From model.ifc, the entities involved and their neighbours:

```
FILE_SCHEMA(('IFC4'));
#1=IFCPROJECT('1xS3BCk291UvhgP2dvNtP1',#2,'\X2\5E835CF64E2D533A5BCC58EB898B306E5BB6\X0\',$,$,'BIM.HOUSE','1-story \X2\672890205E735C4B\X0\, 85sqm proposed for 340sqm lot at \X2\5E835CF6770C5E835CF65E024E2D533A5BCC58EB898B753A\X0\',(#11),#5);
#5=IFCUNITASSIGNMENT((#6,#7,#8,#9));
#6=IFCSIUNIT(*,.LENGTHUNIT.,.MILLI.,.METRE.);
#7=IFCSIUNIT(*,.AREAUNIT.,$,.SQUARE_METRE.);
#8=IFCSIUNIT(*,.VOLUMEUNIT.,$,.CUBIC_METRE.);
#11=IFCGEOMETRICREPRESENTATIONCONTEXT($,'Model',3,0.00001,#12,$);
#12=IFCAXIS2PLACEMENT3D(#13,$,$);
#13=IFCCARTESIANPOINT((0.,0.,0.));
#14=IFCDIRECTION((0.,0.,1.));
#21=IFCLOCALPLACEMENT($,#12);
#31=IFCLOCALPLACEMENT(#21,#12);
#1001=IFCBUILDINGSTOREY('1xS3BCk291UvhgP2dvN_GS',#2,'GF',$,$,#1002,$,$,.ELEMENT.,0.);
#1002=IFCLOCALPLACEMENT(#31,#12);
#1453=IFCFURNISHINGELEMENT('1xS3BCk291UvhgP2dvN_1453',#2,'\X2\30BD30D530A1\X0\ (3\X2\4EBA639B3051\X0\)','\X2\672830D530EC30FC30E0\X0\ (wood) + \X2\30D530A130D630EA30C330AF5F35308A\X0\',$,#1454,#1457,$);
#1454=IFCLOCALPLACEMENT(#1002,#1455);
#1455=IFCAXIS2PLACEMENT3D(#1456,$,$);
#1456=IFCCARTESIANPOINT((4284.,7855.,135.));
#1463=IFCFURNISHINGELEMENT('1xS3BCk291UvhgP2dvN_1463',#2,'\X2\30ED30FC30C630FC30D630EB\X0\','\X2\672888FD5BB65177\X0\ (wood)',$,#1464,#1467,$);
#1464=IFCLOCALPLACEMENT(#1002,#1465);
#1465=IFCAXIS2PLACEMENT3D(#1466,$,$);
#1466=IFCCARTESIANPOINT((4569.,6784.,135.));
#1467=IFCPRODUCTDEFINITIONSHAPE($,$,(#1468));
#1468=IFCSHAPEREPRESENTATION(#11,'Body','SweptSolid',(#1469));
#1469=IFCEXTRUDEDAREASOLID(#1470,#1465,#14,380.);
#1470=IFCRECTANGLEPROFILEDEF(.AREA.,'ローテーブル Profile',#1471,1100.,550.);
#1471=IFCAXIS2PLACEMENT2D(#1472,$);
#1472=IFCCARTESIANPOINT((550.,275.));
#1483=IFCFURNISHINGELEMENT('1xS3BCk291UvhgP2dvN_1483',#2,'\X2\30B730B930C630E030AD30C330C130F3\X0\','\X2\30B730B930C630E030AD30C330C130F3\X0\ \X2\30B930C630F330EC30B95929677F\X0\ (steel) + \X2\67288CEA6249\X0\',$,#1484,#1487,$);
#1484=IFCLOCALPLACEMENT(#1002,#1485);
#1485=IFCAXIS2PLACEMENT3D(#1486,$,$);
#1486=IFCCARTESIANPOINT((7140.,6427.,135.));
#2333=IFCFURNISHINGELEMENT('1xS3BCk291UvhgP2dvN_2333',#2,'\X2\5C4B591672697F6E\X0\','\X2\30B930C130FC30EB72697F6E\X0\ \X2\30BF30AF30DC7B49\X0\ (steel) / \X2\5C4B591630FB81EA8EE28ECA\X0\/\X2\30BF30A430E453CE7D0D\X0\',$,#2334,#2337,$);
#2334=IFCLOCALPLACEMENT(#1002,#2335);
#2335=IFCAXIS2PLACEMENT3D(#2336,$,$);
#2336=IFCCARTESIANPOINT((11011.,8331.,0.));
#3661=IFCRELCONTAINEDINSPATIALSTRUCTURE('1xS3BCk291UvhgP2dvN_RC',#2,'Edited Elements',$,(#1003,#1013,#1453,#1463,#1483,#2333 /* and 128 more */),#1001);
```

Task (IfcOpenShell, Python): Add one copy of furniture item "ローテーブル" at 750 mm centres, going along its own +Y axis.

```python
import ifcopenshell
import ifcopenshell.api.geometry
import ifcopenshell.api.root
import ifcopenshell.util.element
import ifcopenshell.util.placement

model = ifcopenshell.open("model.ifc")


def reuse_history(source, copy):
    """copy_class also copies each property set's owner history, people and application; keep the originals."""
    for rel in copy.IsDefinedBy:
        if rel.is_a("IfcRelDefinesByProperties") and (history := rel.RelatingPropertyDefinition.OwnerHistory):
            rel.RelatingPropertyDefinition.OwnerHistory = source.OwnerHistory
            ifcopenshell.util.element.remove_deep2(model, history)


source = model.by_guid("1xS3BCk291UvhgP2dvN_1463")
base = ifcopenshell.util.placement.get_local_placement(source.ObjectPlacement)
step = base[:3, 1] * 750.0

for i in range(1, 2):
    copy = ifcopenshell.api.root.copy_class(model, product=source)
    copy.Representation = ifcopenshell.util.element.copy_deep(
        model, source.Representation, exclude=["IfcGeometricRepresentationContext", "IfcRepresentationMap"]
    )
    reuse_history(source, copy)
    matrix = base.copy()
    matrix[:3, 3] += i * step
    print("added at", matrix[:3, 3].round(3) + 0.0)
    ifcopenshell.api.geometry.edit_object_placement(model, product=copy, matrix=matrix, is_si=False)

model.write("model_v2.ifc")
```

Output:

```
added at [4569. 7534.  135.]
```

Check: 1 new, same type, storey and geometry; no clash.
